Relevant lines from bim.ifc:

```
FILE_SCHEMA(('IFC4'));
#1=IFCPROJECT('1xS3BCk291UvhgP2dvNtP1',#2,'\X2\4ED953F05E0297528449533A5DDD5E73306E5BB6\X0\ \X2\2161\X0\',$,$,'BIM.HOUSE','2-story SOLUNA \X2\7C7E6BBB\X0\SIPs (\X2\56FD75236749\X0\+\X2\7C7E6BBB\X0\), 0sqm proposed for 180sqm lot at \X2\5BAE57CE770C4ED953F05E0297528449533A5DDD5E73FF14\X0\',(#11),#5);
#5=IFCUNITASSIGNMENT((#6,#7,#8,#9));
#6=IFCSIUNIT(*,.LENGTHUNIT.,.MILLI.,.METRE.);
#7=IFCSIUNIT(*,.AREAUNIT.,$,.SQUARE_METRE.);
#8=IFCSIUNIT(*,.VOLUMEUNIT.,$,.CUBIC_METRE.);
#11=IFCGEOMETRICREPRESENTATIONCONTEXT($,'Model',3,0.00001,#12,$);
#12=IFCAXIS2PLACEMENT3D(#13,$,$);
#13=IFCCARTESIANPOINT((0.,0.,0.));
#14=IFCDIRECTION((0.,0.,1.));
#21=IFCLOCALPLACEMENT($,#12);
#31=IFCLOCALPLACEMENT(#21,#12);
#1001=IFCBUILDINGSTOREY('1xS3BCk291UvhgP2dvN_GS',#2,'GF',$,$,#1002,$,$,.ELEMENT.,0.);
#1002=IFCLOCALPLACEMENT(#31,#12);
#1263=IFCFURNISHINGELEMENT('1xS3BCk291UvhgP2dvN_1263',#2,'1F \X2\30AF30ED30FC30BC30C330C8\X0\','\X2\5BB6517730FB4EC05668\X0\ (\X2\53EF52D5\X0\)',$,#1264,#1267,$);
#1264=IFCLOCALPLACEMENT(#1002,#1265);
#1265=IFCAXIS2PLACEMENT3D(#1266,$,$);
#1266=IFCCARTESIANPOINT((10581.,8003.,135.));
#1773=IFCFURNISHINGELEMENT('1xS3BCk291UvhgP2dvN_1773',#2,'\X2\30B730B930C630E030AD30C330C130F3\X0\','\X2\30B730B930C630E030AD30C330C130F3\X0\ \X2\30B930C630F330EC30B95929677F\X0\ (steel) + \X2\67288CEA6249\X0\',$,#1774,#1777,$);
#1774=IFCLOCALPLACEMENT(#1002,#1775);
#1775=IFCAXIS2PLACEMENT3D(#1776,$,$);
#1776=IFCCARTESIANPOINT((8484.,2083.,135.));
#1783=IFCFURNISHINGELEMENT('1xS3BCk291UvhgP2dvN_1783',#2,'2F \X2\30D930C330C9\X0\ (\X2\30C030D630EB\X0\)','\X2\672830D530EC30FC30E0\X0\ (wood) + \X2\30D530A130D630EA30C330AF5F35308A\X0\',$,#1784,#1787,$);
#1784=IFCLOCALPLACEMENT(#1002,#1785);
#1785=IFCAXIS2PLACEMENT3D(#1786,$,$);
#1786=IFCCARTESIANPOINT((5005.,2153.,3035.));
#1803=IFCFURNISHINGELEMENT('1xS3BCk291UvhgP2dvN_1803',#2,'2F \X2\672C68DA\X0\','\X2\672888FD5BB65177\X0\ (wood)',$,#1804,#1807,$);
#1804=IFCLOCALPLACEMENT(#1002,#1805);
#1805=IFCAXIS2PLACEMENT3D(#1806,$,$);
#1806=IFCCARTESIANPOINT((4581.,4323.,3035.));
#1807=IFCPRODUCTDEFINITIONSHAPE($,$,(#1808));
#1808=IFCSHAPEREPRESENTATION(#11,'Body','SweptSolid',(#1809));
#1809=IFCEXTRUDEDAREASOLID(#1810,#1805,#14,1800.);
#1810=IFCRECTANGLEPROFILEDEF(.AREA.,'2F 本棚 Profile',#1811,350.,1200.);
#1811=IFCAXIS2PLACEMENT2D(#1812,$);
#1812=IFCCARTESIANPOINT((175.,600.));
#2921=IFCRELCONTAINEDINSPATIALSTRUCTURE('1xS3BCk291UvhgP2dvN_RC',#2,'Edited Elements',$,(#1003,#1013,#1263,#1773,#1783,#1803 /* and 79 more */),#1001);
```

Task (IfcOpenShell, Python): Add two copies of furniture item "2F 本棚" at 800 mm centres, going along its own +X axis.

```python
import ifcopenshell
import ifcopenshell.api.geometry
import ifcopenshell.api.root
import ifcopenshell.util.element
import ifcopenshell.util.placement

model = ifcopenshell.open("bim.ifc")


def reuse_history(source, copy):
    """copy_class also copies each property set's owner history, people and application; keep the originals."""
    for rel in copy.IsDefinedBy:
        if rel.is_a("IfcRelDefinesByProperties") and (history := rel.RelatingPropertyDefinition.OwnerHistory):
            rel.RelatingPropertyDefinition.OwnerHistory = source.OwnerHistory
            ifcopenshell.util.element.remove_deep2(model, history)


source = model.by_id(1803)
base = ifcopenshell.util.placement.get_local_placement(source.ObjectPlacement)
step = base[:3, 0] * 800.0

for i in range(1, 3):
    copy = ifcopenshell.api.root.copy_class(model, product=source)
    copy.Representation = ifcopenshell.util.element.copy_deep(
        model, source.Representation, exclude=["IfcGeometricRepresentationContext", "IfcRepresentationMap"]
    )
    reuse_history(source, copy)
    matrix = base.copy()
    matrix[:3, 3] += i * step
    print("added at", matrix[:3, 3].round(3) + 0.0)
    ifcopenshell.api.geometry.edit_object_placement(model, product=copy, matrix=matrix, is_si=False)

model.write("bim_rev.ifc")
```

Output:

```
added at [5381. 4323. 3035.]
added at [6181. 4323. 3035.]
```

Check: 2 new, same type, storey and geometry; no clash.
